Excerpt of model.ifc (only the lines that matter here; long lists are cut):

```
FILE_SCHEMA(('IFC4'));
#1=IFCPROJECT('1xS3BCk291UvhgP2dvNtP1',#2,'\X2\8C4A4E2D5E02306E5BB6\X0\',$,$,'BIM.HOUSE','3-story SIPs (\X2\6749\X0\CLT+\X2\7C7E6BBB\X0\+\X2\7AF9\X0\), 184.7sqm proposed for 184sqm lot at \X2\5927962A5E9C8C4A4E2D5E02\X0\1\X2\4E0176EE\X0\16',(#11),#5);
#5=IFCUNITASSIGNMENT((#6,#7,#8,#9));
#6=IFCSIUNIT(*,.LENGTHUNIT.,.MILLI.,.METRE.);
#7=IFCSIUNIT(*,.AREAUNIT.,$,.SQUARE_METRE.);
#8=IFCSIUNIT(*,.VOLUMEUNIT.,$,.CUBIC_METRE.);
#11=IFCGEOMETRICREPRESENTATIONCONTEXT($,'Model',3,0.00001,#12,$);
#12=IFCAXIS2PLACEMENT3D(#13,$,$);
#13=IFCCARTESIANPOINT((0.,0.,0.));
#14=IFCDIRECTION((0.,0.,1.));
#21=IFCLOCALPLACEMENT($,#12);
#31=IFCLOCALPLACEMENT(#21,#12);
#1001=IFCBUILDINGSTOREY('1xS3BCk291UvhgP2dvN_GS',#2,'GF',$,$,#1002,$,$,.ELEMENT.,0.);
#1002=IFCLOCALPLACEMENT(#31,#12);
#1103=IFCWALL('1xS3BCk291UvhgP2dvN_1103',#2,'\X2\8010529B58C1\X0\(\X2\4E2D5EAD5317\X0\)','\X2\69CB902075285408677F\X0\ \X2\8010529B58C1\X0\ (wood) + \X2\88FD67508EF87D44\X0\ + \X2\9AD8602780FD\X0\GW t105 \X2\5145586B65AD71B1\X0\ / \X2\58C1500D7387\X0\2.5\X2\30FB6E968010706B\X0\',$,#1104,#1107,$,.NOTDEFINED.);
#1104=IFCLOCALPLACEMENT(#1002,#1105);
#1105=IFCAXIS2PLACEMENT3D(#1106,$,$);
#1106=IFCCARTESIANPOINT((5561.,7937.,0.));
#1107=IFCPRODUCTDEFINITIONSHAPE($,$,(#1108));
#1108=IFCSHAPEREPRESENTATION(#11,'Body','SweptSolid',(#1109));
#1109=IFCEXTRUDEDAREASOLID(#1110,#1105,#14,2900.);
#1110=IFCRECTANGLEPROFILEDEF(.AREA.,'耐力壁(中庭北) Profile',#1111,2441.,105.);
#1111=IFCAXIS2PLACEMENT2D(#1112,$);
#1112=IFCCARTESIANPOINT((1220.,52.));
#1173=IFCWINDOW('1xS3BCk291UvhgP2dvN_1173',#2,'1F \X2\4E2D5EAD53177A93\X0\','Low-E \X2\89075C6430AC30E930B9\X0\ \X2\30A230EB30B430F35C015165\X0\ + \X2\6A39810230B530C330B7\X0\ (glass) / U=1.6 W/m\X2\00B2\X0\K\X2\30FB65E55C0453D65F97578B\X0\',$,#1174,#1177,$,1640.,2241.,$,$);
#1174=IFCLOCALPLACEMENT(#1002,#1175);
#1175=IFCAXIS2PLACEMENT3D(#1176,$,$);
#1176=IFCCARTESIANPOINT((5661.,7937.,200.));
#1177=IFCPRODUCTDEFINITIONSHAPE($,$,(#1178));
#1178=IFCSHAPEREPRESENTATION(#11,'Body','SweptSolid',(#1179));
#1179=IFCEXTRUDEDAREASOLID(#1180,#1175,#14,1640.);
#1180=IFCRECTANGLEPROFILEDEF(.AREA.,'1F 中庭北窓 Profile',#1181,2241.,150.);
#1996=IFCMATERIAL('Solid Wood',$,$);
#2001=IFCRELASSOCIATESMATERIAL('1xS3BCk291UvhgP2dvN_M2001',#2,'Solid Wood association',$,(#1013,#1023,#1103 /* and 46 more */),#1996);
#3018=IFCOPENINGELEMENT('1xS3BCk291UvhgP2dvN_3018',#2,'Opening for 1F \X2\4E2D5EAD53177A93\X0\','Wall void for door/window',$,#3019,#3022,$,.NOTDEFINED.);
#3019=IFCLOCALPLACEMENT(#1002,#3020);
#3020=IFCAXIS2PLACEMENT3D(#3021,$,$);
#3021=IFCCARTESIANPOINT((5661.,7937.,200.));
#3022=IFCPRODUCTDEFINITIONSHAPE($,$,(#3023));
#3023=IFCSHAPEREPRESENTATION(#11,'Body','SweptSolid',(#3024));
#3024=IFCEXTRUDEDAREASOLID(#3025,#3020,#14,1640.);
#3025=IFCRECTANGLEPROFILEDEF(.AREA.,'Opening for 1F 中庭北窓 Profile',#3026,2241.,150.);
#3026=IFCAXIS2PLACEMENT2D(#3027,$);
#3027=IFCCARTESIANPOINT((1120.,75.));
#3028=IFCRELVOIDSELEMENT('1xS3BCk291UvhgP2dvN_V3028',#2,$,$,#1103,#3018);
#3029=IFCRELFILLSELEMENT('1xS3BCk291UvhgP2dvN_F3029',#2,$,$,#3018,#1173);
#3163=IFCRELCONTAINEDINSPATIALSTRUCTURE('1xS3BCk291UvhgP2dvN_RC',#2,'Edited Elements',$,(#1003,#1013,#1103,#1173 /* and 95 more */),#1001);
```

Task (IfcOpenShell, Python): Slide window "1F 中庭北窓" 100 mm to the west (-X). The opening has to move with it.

```python
import ifcopenshell
import ifcopenshell.api.geometry
import ifcopenshell.util.placement
import ifcopenshell.util.unit

model = ifcopenshell.open("model.ifc")
unit_scale = ifcopenshell.util.unit.calculate_unit_scale(model)

window = model.by_guid("1xS3BCk291UvhgP2dvN_1173")
opening = window.FillsVoids[0].RelatingOpeningElement
wall = opening.VoidsElements[0].RelatingBuildingElement

wall_matrix = ifcopenshell.util.placement.get_local_placement(wall.ObjectPlacement)
shift = wall_matrix[:3, 0] * -0.1 / unit_scale
before = ifcopenshell.util.placement.get_local_placement(window.ObjectPlacement)[:3, 3].copy()

# The window is not placed relative to its opening, so move both.
for product in (opening, window):
    matrix = ifcopenshell.util.placement.get_local_placement(product.ObjectPlacement)
    matrix[:3, 3] += shift
    ifcopenshell.api.geometry.edit_object_placement(model, product=product, matrix=matrix, is_si=False)

after = ifcopenshell.util.placement.get_local_placement(window.ObjectPlacement)[:3, 3]
print("window moved by", (after - before).round(3) + 0.0)

model.write("model-out.ifc")
```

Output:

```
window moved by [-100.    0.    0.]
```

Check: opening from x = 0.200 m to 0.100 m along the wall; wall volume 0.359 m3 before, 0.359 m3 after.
